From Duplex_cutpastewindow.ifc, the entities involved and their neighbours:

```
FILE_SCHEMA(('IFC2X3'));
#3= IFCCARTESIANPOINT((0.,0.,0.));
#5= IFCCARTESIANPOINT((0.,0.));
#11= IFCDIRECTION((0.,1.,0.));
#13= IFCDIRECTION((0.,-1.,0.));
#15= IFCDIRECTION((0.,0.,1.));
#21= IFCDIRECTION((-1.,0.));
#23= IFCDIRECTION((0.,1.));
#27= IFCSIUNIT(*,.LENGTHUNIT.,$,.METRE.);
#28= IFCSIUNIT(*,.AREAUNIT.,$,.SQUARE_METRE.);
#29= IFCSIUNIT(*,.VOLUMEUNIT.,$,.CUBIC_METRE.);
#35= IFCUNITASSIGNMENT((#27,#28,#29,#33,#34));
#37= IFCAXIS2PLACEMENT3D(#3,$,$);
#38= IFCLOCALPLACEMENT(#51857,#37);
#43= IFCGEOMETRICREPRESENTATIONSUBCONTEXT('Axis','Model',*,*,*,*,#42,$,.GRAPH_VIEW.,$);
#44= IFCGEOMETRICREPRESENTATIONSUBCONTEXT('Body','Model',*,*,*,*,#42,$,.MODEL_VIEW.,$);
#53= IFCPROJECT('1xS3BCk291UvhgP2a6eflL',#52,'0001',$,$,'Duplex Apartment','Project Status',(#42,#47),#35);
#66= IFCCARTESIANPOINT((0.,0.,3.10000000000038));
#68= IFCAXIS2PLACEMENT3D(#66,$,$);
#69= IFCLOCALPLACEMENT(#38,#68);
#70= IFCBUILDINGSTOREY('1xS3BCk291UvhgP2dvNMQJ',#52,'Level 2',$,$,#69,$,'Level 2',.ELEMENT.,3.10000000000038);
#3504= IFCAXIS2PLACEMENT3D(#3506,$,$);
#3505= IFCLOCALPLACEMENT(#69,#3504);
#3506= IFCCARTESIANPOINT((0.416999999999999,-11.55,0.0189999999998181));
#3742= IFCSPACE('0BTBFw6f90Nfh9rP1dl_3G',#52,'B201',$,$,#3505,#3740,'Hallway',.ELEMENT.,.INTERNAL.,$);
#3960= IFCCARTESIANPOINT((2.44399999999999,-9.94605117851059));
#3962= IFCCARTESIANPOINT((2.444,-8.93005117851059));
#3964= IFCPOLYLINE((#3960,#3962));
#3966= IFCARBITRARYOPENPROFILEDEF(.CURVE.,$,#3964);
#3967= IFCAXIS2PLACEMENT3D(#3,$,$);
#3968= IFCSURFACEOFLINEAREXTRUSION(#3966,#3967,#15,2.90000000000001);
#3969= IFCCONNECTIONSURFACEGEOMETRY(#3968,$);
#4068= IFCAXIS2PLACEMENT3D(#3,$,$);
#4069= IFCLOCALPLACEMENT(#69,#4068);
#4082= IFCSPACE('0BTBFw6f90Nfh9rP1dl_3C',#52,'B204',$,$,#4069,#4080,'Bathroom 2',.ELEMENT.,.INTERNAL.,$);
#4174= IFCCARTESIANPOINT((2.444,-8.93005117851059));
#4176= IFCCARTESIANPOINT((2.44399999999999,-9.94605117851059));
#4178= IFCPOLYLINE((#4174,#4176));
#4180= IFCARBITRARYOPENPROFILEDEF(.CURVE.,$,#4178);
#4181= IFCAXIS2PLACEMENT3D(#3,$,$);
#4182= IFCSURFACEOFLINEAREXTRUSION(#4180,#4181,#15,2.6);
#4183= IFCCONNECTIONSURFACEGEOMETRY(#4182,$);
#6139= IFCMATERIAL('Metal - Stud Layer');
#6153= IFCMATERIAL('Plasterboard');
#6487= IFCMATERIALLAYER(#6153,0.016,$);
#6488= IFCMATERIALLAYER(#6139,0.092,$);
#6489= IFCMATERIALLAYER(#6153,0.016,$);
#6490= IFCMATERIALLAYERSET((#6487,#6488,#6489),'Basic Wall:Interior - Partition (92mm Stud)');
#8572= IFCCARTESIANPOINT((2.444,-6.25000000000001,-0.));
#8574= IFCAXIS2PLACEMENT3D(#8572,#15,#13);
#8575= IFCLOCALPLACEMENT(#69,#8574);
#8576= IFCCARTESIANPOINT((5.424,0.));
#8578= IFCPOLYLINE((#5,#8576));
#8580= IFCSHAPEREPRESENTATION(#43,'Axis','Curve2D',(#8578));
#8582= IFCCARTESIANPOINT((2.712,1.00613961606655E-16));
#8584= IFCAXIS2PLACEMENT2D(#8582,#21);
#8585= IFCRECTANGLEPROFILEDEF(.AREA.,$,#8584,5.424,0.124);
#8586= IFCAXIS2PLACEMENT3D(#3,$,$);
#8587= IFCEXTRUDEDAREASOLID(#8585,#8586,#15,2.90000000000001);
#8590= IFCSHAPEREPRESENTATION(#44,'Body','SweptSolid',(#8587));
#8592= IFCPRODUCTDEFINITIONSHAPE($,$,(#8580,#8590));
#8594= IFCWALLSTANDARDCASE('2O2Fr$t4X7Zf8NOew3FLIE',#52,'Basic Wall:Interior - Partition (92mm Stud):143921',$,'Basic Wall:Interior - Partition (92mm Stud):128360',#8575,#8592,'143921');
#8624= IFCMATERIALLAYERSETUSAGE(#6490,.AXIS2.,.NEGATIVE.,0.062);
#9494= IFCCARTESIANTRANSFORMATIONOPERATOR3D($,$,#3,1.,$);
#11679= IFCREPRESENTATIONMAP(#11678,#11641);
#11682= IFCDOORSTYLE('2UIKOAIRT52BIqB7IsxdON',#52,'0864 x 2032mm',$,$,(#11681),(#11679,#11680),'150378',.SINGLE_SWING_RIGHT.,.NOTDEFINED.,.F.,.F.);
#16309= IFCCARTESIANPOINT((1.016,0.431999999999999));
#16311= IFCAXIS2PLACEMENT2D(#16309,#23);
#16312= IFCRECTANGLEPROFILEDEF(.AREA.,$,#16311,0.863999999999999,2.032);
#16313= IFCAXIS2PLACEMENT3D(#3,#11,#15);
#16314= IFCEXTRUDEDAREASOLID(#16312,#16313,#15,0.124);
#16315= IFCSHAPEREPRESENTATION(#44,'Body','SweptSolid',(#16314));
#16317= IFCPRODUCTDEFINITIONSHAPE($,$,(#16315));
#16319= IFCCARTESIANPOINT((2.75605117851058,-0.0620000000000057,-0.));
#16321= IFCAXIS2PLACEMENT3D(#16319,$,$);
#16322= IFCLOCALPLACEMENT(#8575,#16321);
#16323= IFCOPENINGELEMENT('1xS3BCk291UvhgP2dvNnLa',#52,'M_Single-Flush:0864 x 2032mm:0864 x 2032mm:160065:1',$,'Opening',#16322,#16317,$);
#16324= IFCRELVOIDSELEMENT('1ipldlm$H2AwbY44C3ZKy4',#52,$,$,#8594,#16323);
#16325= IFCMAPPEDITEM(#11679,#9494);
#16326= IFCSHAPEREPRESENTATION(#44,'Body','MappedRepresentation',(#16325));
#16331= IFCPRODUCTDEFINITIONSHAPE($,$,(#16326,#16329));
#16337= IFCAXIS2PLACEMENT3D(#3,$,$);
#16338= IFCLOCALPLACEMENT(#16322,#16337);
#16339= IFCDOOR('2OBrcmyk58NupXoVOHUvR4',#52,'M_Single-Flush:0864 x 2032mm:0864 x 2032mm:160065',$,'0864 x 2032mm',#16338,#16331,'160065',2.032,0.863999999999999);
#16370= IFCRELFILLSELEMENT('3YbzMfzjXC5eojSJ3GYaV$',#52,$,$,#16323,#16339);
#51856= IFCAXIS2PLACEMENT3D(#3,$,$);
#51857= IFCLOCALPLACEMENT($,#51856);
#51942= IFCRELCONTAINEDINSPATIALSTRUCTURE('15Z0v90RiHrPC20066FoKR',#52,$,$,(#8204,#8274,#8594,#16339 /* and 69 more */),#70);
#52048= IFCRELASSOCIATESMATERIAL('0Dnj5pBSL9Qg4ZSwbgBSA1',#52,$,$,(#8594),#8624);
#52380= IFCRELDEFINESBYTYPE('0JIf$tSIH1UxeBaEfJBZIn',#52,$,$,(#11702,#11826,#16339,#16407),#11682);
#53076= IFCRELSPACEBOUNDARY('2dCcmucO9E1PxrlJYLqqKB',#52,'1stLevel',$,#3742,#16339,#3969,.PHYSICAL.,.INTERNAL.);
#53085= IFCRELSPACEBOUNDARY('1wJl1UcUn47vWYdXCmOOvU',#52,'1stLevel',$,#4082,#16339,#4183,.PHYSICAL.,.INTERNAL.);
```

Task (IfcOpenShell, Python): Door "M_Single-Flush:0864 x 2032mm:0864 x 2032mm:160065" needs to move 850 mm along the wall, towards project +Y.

```python
import numpy as np
import ifcopenshell
import ifcopenshell.api.geometry
import ifcopenshell.util.placement
import ifcopenshell.util.unit

model = ifcopenshell.open("Duplex_cutpastewindow.ifc")
unit_scale = ifcopenshell.util.unit.calculate_unit_scale(model)

door = model.by_guid("2OBrcmyk58NupXoVOHUvR4")
opening = door.FillsVoids[0].RelatingOpeningElement
wall = opening.VoidsElements[0].RelatingBuildingElement

wall_matrix = ifcopenshell.util.placement.get_local_placement(wall.ObjectPlacement)
shift = wall_matrix[:3, 0] * -0.85 / unit_scale
before = ifcopenshell.util.placement.get_local_placement(door.ObjectPlacement)[:3, 3].copy()

# The door is placed relative to its opening, so it follows when the opening moves.
matrix = ifcopenshell.util.placement.get_local_placement(opening.ObjectPlacement)
matrix[:3, 3] += shift
ifcopenshell.api.geometry.edit_object_placement(
    model, product=opening, matrix=matrix, is_si=False, should_transform_children=True
)

# Space boundary surfaces are stored in each space's coordinates; move them too.
for rel in door.ProvidesBoundaries:
    if not rel.ConnectionGeometry:
        continue
    surface = rel.ConnectionGeometry.SurfaceOnRelatingElement
    space_matrix = ifcopenshell.util.placement.get_local_placement(rel.RelatingSpace.ObjectPlacement)
    point = np.array(surface.Position.Location.Coordinates) + space_matrix[:3, :3].T @ shift
    surface.Position = model.createIfcAxis2Placement3D(
        model.createIfcCartesianPoint(point.tolist()), surface.Position.Axis, surface.Position.RefDirection
    )

after = ifcopenshell.util.placement.get_local_placement(door.ObjectPlacement)[:3, 3]
print("door moved by", (after - before).round(3) + 0.0)

model.write("Duplex_cutpastewindow_updated.ifc")
```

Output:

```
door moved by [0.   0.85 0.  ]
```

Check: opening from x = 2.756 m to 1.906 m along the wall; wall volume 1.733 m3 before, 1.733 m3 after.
